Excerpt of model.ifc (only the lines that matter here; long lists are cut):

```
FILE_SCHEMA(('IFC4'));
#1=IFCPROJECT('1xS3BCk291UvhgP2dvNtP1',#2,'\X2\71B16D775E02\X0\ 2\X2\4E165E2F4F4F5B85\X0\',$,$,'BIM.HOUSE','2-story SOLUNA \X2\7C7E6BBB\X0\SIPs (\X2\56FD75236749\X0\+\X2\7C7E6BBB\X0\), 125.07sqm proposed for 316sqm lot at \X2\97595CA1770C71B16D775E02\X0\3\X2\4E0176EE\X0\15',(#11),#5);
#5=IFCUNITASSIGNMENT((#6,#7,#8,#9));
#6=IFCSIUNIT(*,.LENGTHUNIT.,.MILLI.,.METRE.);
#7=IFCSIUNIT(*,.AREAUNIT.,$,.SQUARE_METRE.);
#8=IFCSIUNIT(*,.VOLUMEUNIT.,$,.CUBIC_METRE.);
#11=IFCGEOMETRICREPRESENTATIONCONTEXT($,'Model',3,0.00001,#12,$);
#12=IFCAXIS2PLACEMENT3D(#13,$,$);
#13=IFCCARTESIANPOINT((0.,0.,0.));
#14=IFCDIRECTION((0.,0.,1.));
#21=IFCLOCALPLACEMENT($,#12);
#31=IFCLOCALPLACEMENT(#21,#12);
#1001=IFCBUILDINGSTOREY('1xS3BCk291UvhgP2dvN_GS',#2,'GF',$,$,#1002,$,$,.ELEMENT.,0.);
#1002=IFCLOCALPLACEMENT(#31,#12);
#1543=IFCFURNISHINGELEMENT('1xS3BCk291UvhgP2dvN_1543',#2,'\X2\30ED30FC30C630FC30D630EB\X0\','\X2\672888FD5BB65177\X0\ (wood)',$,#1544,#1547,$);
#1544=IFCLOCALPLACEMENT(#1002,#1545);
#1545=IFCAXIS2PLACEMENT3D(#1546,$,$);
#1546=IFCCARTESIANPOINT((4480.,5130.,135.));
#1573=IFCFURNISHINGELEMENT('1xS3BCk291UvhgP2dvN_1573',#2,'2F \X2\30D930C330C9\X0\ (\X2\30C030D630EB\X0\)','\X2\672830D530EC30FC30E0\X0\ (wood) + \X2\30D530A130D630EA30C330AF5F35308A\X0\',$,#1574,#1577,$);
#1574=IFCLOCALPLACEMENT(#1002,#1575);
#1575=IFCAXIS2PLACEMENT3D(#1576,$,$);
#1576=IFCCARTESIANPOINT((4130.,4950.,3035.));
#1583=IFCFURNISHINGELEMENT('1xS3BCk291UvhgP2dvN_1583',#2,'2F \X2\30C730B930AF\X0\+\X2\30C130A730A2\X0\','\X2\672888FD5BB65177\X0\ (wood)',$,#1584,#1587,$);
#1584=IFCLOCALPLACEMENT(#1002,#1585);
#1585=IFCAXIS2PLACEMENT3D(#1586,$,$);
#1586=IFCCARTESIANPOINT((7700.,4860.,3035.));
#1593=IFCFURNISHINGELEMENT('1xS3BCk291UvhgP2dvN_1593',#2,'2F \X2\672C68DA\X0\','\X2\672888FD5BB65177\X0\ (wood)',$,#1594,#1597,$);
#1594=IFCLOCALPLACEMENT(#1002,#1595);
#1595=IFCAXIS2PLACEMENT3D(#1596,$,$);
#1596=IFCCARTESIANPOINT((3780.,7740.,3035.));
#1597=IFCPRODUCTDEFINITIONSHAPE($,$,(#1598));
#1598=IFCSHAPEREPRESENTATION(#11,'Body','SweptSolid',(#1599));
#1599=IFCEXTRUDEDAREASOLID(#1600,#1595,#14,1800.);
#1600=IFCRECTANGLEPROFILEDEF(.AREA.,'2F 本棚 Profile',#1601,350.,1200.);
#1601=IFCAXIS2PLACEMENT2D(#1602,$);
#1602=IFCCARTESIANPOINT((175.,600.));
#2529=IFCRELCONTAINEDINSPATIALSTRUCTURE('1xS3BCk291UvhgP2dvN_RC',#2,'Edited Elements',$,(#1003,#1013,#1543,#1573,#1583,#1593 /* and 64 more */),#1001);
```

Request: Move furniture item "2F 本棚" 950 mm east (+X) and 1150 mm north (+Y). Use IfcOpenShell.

```python
import ifcopenshell
import ifcopenshell.api.geometry
import ifcopenshell.util.placement
import ifcopenshell.util.unit

model = ifcopenshell.open("model.ifc")
unit_scale = ifcopenshell.util.unit.calculate_unit_scale(model)

item = model.by_id(1593)
matrix = ifcopenshell.util.placement.get_local_placement(item.ObjectPlacement)
matrix[0, 3] += 0.95 / unit_scale
matrix[1, 3] += 1.15 / unit_scale
ifcopenshell.api.geometry.edit_object_placement(model, product=item, matrix=matrix, is_si=False)

print(ifcopenshell.util.placement.get_local_placement(item.ObjectPlacement).round(3) + 0.0)

model.write("model_v2.ifc")
```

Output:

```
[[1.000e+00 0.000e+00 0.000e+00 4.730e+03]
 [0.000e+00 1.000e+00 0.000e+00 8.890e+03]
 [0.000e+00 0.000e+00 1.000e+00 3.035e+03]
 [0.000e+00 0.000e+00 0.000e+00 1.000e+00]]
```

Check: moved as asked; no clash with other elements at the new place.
